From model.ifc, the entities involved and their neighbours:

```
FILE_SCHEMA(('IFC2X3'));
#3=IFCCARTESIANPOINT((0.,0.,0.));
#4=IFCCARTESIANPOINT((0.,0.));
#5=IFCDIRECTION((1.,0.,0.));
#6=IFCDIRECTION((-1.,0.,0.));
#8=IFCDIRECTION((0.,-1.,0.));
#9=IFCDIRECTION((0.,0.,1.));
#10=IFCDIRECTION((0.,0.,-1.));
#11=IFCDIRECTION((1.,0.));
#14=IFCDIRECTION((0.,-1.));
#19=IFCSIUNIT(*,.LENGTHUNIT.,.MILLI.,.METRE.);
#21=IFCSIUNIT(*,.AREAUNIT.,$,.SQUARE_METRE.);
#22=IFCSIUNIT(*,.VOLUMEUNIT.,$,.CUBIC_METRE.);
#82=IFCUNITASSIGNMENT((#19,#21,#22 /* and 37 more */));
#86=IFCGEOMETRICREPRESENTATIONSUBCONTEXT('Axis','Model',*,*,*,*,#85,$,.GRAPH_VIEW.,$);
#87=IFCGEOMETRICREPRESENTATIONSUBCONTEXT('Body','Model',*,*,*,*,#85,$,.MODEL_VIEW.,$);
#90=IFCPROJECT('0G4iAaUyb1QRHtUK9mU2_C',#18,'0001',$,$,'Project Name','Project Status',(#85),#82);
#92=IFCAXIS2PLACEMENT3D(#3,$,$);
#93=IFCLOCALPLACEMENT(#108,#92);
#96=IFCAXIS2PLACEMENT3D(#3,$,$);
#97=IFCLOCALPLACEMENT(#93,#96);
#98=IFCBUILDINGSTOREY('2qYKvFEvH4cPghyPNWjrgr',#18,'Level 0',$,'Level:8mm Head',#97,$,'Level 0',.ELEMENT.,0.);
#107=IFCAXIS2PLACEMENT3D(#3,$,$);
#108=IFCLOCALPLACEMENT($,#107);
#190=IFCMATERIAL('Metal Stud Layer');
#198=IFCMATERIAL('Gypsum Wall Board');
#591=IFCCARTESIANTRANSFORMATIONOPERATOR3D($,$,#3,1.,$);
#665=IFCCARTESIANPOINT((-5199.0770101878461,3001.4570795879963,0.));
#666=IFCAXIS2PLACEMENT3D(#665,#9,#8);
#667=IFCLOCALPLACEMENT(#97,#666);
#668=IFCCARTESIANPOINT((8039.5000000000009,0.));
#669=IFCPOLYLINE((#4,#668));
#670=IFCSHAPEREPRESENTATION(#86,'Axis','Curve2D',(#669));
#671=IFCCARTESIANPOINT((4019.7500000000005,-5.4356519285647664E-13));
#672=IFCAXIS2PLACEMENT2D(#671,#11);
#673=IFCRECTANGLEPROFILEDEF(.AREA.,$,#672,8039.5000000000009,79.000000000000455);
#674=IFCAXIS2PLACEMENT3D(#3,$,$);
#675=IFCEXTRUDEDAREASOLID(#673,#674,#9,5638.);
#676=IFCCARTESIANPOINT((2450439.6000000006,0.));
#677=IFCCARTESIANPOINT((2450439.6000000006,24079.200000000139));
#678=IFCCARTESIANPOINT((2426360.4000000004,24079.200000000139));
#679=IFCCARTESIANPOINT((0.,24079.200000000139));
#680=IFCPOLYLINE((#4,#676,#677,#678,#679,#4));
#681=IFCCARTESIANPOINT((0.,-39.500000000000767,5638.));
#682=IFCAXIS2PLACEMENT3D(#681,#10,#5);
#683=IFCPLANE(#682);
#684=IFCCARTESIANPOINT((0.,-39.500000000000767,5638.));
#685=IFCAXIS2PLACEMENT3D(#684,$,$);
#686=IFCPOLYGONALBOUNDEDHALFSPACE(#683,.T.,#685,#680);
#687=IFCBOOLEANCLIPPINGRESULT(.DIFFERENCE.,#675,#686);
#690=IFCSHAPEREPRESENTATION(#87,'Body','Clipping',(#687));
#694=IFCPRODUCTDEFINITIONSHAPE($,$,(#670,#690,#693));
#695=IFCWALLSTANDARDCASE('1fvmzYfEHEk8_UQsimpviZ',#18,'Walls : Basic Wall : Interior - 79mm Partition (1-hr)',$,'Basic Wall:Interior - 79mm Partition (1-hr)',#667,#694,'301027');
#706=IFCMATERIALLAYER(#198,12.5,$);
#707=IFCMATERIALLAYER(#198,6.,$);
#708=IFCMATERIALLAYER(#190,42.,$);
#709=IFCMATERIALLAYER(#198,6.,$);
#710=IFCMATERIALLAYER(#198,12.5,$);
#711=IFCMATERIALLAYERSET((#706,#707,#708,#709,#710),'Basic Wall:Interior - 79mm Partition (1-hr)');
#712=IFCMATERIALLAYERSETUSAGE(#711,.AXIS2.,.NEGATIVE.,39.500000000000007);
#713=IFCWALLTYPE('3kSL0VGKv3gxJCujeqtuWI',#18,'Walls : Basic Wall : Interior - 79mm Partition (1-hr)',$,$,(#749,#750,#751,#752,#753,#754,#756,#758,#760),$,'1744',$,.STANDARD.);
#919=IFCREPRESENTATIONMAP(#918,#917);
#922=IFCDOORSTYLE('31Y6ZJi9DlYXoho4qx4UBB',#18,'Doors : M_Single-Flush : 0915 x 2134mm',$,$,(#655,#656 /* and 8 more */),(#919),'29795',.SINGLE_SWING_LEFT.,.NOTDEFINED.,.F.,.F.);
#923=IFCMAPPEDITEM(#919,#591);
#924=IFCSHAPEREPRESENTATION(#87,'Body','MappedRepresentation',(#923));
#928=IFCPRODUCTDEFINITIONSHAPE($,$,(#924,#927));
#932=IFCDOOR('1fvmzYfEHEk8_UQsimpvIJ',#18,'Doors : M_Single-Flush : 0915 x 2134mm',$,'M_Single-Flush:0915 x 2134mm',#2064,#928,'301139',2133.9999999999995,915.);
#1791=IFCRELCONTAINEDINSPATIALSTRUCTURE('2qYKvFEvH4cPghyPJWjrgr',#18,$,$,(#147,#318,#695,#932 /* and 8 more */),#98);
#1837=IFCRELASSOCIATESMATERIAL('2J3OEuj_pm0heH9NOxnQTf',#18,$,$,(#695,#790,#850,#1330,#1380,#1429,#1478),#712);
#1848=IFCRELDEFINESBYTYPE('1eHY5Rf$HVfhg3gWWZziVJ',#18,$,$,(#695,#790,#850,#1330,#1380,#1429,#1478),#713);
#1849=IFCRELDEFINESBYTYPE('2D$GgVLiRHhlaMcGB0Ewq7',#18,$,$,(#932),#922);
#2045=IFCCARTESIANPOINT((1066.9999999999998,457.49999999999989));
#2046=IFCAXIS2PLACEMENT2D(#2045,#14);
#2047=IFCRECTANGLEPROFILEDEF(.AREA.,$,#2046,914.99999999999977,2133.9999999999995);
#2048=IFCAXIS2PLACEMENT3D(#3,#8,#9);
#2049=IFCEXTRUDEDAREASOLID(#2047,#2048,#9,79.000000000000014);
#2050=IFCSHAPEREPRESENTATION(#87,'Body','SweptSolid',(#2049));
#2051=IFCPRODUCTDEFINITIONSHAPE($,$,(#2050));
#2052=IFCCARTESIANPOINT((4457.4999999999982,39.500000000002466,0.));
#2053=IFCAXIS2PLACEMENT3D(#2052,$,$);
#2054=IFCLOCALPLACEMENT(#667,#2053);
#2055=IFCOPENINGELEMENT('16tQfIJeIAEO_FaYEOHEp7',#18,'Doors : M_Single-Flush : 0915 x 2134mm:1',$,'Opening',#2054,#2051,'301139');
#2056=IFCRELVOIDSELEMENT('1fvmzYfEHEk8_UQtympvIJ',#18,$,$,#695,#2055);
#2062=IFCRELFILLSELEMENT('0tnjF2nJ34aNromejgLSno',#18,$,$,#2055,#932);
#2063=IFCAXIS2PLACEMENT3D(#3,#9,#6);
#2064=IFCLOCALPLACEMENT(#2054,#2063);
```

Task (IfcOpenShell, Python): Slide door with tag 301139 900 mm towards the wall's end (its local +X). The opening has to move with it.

```python
import ifcopenshell
import ifcopenshell.api.geometry
import ifcopenshell.util.placement
import ifcopenshell.util.unit

model = ifcopenshell.open("model.ifc")
unit_scale = ifcopenshell.util.unit.calculate_unit_scale(model)

door = model.by_guid("1fvmzYfEHEk8_UQsimpvIJ")
opening = door.FillsVoids[0].RelatingOpeningElement
wall = opening.VoidsElements[0].RelatingBuildingElement

wall_matrix = ifcopenshell.util.placement.get_local_placement(wall.ObjectPlacement)
shift = wall_matrix[:3, 0] * 0.9 / unit_scale
before = ifcopenshell.util.placement.get_local_placement(door.ObjectPlacement)[:3, 3].copy()

# The door is placed relative to its opening, so it follows when the opening moves.
matrix = ifcopenshell.util.placement.get_local_placement(opening.ObjectPlacement)
matrix[:3, 3] += shift
ifcopenshell.api.geometry.edit_object_placement(
    model, product=opening, matrix=matrix, is_si=False, should_transform_children=True
)

after = ifcopenshell.util.placement.get_local_placement(door.ObjectPlacement)[:3, 3]
print("door moved by", (after - before).round(3) + 0.0)

model.write("model_rev.ifc")
```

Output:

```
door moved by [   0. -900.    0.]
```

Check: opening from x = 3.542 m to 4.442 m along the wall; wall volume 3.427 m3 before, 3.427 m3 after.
